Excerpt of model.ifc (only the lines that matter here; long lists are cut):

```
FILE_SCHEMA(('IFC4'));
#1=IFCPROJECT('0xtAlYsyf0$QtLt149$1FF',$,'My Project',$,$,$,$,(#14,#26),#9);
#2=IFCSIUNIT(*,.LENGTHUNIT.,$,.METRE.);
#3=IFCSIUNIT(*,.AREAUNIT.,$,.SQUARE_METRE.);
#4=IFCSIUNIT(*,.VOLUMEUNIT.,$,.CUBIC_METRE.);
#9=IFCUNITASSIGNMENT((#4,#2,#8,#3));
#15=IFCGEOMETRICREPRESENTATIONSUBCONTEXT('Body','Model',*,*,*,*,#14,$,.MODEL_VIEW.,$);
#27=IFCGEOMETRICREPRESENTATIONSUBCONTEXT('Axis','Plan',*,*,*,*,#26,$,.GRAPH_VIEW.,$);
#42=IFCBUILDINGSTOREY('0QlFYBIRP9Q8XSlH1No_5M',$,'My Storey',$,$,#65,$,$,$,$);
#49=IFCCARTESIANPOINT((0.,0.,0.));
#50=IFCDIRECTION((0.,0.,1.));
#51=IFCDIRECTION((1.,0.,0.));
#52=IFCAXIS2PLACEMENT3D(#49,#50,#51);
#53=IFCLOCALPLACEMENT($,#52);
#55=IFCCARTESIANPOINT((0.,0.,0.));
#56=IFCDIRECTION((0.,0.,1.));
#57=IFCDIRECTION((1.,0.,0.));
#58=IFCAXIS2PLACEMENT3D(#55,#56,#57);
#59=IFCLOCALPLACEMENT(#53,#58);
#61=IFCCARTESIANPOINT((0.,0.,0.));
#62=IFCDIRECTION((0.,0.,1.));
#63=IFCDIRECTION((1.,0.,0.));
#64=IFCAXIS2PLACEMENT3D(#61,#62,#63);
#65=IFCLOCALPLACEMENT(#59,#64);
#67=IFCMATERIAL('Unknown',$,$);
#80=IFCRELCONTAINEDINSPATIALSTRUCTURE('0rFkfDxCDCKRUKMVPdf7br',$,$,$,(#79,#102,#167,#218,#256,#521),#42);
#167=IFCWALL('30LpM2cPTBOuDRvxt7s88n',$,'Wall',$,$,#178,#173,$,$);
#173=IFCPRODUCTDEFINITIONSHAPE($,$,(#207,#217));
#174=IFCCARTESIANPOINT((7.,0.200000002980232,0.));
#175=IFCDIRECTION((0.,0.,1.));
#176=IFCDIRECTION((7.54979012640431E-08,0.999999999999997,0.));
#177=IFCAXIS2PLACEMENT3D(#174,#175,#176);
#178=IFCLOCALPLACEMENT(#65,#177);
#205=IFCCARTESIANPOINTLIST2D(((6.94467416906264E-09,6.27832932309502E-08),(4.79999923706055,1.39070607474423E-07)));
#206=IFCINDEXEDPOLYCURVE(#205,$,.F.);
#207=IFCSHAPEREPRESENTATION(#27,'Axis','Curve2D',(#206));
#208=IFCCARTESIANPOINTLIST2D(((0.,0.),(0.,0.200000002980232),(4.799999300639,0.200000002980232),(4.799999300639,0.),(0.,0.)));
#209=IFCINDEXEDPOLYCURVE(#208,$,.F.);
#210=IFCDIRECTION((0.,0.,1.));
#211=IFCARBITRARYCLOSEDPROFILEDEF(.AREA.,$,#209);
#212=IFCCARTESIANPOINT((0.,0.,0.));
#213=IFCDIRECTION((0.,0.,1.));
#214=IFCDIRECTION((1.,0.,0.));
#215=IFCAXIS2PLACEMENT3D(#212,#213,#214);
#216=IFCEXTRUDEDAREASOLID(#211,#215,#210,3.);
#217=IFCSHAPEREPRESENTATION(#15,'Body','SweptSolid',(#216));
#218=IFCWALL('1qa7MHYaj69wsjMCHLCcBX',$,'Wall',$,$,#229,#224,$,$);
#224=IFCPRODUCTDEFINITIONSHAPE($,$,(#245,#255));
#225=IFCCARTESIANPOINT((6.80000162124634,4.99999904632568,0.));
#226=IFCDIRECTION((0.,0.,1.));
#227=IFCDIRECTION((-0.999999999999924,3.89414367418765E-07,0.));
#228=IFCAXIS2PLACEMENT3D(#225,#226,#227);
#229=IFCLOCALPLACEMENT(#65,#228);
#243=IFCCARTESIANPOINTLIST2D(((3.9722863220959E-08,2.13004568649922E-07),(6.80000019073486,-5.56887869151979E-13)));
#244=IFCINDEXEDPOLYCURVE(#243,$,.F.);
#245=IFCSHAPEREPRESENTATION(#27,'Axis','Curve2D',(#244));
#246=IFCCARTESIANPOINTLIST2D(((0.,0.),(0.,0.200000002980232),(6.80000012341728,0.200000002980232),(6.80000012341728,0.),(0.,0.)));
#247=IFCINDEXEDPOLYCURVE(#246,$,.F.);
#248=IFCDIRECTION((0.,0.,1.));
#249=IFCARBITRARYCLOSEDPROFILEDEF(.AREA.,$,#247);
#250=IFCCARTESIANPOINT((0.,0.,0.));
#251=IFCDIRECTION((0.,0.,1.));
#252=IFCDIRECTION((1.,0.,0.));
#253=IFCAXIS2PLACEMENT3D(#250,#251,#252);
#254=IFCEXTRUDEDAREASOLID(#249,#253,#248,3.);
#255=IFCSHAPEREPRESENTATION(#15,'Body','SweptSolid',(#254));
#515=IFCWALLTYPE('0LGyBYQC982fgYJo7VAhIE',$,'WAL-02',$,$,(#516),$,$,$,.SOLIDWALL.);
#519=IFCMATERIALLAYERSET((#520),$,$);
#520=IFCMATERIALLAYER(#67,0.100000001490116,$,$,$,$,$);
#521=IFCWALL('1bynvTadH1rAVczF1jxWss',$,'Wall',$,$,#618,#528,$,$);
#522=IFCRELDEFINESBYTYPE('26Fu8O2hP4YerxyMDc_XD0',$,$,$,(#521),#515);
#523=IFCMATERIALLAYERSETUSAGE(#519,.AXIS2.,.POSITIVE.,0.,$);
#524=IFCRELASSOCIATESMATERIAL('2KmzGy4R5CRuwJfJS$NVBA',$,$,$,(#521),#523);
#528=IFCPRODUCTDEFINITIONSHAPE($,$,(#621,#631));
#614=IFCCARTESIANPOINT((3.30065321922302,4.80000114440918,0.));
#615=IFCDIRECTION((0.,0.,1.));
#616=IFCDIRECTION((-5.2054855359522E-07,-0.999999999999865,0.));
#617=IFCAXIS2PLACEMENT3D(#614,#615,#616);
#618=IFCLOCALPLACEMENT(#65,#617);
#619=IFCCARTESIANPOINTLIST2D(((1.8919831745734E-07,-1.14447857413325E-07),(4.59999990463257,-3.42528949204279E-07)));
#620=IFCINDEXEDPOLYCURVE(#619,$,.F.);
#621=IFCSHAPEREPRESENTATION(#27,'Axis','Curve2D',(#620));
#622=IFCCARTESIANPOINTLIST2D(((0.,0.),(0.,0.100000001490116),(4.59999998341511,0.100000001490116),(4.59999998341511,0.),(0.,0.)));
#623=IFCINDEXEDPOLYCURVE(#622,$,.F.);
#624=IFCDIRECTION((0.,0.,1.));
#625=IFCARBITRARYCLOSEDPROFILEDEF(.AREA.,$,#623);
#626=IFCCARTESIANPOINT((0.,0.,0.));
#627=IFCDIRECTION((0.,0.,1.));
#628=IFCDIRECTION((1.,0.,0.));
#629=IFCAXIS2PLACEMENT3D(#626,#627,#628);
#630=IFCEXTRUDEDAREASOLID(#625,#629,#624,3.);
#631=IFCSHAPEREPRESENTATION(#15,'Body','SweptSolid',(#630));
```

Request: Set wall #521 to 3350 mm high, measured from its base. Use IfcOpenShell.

```python
import ifcopenshell
import ifcopenshell.geom
import ifcopenshell.util.representation
import ifcopenshell.util.shape
import ifcopenshell.util.unit

model = ifcopenshell.open("model.ifc")
unit_scale = ifcopenshell.util.unit.calculate_unit_scale(model)
settings = ifcopenshell.geom.settings()


def volume(element):
    """Net volume in cubic metres, openings subtracted."""
    shape = ifcopenshell.geom.create_shape(settings, element)
    return ifcopenshell.util.shape.get_volume(shape.geometry)


wall = model.by_guid("1bynvTadH1rAVczF1jxWss")
before = volume(wall)

body = ifcopenshell.util.representation.get_representation(wall, "Model", "Body")
solid = body.Items[0]
old_height = solid.Depth
solid.Depth = 3.35 / unit_scale
after = volume(wall)

print(f"height {old_height:g} -> {solid.Depth:g}, volume {before:.3f} -> {after:.3f} m3")

model.write("model_v2.ifc")
```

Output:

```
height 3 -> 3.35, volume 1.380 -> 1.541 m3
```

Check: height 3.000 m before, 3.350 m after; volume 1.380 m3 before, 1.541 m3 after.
